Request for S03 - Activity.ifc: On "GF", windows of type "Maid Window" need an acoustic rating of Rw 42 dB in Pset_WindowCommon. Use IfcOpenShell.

First a look at what the model holds.

```python
import ifcopenshell
import ifcopenshell.util.element

model = ifcopenshell.open("S03 - Activity.ifc")
print(model.schema)
storey = next(s for s in model.by_type("IfcBuildingStorey") if s.Name == "GF")
windows = [e for e in ifcopenshell.util.element.get_decomposition(storey) if e.is_a("IfcWindow")]
seen = {}
for e in windows:
    element_type = ifcopenshell.util.element.get_type(e)
    key = (element_type.Name if element_type != e and element_type else None, ifcopenshell.util.element.get_pset(e, "Pset_WindowCommon", "AcousticRating"))
    seen[key] = seen.get(key, 0) + 1
for (name, value), count in sorted(seen.items(), key=str):
    print(count, "x", name, "|", value)
```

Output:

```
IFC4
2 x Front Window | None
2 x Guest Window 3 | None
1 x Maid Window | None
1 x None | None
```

```python
import ifcopenshell
import ifcopenshell.api.pset
import ifcopenshell.util.element

model = ifcopenshell.open("S03 - Activity.ifc")

storey = next(s for s in model.by_type("IfcBuildingStorey") if s.Name == "GF")
windows = [e for e in ifcopenshell.util.element.get_decomposition(storey) if e.is_a("IfcWindow")]

count = 0
for e in windows:
    element_type = ifcopenshell.util.element.get_type(e)
    if element_type in (None, e) or element_type.Name != "Maid Window":
        continue
    # add_pset returns the element's existing set when there is one.
    pset = ifcopenshell.api.pset.add_pset(model, product=e, name="Pset_WindowCommon")
    ifcopenshell.api.pset.edit_pset(model, pset=pset, properties={"AcousticRating": "Rw 42 dB"})
    count += 1

print(count, "windows updated")

model.write("S03 - Activity-out.ifc")
```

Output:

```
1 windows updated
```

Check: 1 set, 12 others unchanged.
